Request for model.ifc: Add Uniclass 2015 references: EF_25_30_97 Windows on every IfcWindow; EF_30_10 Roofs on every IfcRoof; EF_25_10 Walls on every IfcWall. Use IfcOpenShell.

First a look at what the model holds.

```python
import ifcopenshell

model = ifcopenshell.open("model.ifc")
print(model.schema)
print("classifications:", [c.Name for c in model.by_type("IfcClassification")])
for ifc_class in ("IfcDoor", "IfcRoof", "IfcStair", "IfcWall", "IfcWindow"):
    print(ifc_class, len(model.by_type(ifc_class)))
```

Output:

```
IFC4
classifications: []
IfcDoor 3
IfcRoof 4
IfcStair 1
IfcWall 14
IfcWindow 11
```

```python
import ifcopenshell
import ifcopenshell.api.classification

model = ifcopenshell.open("model.ifc")

system = ifcopenshell.api.classification.add_classification(model, classification="Uniclass 2015")

codes = {
    "IfcWindow": ("EF_25_30_97", "Windows"),
    "IfcRoof": ("EF_30_10", "Roofs"),
    "IfcWall": ("EF_25_10", "Walls"),
}
for ifc_class, (code, name) in codes.items():
    products = model.by_type(ifc_class)
    ifcopenshell.api.classification.add_reference(
        model, products=products, classification=system, identification=code, name=name
    )
    print(code, len(products))

model.write("model-out.ifc")
```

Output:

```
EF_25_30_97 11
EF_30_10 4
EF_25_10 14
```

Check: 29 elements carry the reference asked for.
